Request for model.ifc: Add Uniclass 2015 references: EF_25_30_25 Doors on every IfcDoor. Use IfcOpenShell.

First a look at what the model holds.

```python
import ifcopenshell

model = ifcopenshell.open("model.ifc")
print(model.schema)
print("classifications:", [c.Name for c in model.by_type("IfcClassification")])
for ifc_class in ("IfcDoor", "IfcRoof", "IfcStair", "IfcWall", "IfcWindow"):
    print(ifc_class, len(model.by_type(ifc_class)))
```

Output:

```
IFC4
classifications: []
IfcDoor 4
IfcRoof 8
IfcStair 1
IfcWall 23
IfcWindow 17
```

```python
import ifcopenshell
import ifcopenshell.api.classification

model = ifcopenshell.open("model.ifc")

system = ifcopenshell.api.classification.add_classification(model, classification="Uniclass 2015")

codes = {
    "IfcDoor": ("EF_25_30_25", "Doors"),
}
for ifc_class, (code, name) in codes.items():
    products = model.by_type(ifc_class)
    ifcopenshell.api.classification.add_reference(
        model, products=products, classification=system, identification=code, name=name
    )
    print(code, len(products))

model.write("model_edited.ifc")
```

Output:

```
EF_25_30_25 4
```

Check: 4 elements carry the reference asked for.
